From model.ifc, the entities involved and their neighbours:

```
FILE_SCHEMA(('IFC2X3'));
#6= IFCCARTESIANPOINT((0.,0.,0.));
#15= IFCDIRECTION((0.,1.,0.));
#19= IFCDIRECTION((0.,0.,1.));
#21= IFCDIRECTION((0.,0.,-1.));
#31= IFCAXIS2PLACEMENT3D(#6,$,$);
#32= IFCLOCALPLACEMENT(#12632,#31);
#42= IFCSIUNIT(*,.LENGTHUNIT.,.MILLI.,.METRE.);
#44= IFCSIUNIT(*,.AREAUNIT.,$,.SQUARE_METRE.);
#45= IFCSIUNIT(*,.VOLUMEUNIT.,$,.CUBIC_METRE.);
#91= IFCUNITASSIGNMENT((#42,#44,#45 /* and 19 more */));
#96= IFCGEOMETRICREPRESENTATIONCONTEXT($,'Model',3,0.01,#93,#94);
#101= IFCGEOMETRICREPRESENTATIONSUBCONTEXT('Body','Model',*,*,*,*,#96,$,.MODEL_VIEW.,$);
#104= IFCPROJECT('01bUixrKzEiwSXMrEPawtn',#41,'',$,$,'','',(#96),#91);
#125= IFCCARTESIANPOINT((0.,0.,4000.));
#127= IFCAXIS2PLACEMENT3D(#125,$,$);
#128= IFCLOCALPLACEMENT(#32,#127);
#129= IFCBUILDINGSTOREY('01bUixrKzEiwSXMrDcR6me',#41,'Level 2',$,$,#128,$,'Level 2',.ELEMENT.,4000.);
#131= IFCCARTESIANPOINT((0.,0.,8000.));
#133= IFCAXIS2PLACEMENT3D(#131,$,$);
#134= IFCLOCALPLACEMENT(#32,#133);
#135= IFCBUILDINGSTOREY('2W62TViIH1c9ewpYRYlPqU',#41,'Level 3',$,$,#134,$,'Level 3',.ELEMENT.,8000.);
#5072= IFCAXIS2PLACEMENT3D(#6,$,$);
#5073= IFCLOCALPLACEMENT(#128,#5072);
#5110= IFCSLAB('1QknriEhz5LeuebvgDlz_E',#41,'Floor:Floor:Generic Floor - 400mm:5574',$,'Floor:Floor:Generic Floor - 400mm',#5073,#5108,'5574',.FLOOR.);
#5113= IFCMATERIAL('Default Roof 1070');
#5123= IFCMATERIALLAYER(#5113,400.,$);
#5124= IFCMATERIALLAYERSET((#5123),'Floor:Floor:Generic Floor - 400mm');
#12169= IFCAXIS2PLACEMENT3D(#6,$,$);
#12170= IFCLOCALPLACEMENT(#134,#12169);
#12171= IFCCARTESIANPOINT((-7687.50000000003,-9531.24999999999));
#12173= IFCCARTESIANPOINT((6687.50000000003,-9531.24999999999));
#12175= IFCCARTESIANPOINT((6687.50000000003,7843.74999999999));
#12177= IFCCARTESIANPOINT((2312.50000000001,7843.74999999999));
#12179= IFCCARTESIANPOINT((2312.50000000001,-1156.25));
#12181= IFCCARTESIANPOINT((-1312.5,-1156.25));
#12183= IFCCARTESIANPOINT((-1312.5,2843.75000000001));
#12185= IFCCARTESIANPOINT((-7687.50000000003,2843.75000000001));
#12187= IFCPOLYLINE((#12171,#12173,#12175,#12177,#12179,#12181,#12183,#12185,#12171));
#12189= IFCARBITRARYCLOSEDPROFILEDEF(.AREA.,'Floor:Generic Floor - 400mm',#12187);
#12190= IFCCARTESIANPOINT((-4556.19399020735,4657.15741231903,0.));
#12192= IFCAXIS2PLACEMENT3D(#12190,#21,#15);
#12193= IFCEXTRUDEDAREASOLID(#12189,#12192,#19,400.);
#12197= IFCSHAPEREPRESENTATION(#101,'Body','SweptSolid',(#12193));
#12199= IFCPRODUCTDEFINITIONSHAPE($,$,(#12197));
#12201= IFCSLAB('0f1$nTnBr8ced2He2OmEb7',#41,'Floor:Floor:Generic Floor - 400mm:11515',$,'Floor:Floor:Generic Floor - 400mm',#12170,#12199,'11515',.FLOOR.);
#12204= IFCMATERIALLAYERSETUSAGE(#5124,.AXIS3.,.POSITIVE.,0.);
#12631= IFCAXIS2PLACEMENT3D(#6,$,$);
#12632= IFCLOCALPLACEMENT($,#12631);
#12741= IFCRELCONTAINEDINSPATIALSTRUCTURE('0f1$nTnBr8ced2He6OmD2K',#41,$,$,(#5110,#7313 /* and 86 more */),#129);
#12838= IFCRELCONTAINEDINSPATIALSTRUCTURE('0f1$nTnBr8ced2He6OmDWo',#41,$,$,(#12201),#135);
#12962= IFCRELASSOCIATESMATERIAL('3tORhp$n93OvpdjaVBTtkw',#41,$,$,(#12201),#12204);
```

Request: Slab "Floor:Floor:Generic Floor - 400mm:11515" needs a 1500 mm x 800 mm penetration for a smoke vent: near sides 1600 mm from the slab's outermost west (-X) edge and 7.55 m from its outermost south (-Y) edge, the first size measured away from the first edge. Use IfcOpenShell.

```python
import numpy as np
import ifcopenshell
import ifcopenshell.api.feature
import ifcopenshell.api.geometry
import ifcopenshell.api.root
import ifcopenshell.geom
import ifcopenshell.util.placement
import ifcopenshell.util.representation
import ifcopenshell.util.shape
import ifcopenshell.util.unit

model = ifcopenshell.open("model.ifc")
unit_scale = ifcopenshell.util.unit.calculate_unit_scale(model)
settings = ifcopenshell.geom.settings()


def volume(element):
    """Net volume in cubic metres, openings subtracted."""
    shape = ifcopenshell.geom.create_shape(settings, element)
    return ifcopenshell.util.shape.get_volume(shape.geometry)


slab = model.by_guid("0f1$nTnBr8ced2He2OmEb7")
before = volume(slab)

# Extent in the slab's own axes, in metres. The edges named are its -X and -Y sides.
slab_shape = ifcopenshell.geom.create_shape(settings, slab)
vertices = ifcopenshell.util.shape.get_vertices(slab_shape.geometry)
x_min, y_min, bottom = vertices.min(axis=0)
top = vertices[:, 2].max()

opening = ifcopenshell.api.root.create_entity(model, ifc_class="IfcOpeningElement", name="Smoke vent opening")
context = ifcopenshell.util.representation.get_context(model, "Model", "Body", "MODEL_VIEW")
width, depth = 1.5, 0.8
outline = [(0.0, 0.0), (width, 0.0), (width, depth), (0.0, depth), (0.0, 0.0)]
# Overshoot both faces by 50 mm so the cut is clean.
shape = ifcopenshell.api.geometry.add_slab_representation(
    model, context=context, depth=top - bottom + 0.1, polyline=outline
)
ifcopenshell.api.geometry.assign_representation(model, product=opening, representation=shape)

matrix = ifcopenshell.util.placement.get_local_placement(slab.ObjectPlacement)
matrix[:, 3] = matrix @ np.append(np.array([x_min + 1.6, y_min + 7.55, bottom - 0.05]) / unit_scale, 1.0)
ifcopenshell.api.geometry.edit_object_placement(model, product=opening, matrix=matrix, is_si=False)
ifcopenshell.api.feature.add_feature(model, feature=opening, element=slab)

after = volume(slab)

print(f"slab volume {before:.3f} -> {after:.3f} m3")

model.write("model_updated.ifc")
```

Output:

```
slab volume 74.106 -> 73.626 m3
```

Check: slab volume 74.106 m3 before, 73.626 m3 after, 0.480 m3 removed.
